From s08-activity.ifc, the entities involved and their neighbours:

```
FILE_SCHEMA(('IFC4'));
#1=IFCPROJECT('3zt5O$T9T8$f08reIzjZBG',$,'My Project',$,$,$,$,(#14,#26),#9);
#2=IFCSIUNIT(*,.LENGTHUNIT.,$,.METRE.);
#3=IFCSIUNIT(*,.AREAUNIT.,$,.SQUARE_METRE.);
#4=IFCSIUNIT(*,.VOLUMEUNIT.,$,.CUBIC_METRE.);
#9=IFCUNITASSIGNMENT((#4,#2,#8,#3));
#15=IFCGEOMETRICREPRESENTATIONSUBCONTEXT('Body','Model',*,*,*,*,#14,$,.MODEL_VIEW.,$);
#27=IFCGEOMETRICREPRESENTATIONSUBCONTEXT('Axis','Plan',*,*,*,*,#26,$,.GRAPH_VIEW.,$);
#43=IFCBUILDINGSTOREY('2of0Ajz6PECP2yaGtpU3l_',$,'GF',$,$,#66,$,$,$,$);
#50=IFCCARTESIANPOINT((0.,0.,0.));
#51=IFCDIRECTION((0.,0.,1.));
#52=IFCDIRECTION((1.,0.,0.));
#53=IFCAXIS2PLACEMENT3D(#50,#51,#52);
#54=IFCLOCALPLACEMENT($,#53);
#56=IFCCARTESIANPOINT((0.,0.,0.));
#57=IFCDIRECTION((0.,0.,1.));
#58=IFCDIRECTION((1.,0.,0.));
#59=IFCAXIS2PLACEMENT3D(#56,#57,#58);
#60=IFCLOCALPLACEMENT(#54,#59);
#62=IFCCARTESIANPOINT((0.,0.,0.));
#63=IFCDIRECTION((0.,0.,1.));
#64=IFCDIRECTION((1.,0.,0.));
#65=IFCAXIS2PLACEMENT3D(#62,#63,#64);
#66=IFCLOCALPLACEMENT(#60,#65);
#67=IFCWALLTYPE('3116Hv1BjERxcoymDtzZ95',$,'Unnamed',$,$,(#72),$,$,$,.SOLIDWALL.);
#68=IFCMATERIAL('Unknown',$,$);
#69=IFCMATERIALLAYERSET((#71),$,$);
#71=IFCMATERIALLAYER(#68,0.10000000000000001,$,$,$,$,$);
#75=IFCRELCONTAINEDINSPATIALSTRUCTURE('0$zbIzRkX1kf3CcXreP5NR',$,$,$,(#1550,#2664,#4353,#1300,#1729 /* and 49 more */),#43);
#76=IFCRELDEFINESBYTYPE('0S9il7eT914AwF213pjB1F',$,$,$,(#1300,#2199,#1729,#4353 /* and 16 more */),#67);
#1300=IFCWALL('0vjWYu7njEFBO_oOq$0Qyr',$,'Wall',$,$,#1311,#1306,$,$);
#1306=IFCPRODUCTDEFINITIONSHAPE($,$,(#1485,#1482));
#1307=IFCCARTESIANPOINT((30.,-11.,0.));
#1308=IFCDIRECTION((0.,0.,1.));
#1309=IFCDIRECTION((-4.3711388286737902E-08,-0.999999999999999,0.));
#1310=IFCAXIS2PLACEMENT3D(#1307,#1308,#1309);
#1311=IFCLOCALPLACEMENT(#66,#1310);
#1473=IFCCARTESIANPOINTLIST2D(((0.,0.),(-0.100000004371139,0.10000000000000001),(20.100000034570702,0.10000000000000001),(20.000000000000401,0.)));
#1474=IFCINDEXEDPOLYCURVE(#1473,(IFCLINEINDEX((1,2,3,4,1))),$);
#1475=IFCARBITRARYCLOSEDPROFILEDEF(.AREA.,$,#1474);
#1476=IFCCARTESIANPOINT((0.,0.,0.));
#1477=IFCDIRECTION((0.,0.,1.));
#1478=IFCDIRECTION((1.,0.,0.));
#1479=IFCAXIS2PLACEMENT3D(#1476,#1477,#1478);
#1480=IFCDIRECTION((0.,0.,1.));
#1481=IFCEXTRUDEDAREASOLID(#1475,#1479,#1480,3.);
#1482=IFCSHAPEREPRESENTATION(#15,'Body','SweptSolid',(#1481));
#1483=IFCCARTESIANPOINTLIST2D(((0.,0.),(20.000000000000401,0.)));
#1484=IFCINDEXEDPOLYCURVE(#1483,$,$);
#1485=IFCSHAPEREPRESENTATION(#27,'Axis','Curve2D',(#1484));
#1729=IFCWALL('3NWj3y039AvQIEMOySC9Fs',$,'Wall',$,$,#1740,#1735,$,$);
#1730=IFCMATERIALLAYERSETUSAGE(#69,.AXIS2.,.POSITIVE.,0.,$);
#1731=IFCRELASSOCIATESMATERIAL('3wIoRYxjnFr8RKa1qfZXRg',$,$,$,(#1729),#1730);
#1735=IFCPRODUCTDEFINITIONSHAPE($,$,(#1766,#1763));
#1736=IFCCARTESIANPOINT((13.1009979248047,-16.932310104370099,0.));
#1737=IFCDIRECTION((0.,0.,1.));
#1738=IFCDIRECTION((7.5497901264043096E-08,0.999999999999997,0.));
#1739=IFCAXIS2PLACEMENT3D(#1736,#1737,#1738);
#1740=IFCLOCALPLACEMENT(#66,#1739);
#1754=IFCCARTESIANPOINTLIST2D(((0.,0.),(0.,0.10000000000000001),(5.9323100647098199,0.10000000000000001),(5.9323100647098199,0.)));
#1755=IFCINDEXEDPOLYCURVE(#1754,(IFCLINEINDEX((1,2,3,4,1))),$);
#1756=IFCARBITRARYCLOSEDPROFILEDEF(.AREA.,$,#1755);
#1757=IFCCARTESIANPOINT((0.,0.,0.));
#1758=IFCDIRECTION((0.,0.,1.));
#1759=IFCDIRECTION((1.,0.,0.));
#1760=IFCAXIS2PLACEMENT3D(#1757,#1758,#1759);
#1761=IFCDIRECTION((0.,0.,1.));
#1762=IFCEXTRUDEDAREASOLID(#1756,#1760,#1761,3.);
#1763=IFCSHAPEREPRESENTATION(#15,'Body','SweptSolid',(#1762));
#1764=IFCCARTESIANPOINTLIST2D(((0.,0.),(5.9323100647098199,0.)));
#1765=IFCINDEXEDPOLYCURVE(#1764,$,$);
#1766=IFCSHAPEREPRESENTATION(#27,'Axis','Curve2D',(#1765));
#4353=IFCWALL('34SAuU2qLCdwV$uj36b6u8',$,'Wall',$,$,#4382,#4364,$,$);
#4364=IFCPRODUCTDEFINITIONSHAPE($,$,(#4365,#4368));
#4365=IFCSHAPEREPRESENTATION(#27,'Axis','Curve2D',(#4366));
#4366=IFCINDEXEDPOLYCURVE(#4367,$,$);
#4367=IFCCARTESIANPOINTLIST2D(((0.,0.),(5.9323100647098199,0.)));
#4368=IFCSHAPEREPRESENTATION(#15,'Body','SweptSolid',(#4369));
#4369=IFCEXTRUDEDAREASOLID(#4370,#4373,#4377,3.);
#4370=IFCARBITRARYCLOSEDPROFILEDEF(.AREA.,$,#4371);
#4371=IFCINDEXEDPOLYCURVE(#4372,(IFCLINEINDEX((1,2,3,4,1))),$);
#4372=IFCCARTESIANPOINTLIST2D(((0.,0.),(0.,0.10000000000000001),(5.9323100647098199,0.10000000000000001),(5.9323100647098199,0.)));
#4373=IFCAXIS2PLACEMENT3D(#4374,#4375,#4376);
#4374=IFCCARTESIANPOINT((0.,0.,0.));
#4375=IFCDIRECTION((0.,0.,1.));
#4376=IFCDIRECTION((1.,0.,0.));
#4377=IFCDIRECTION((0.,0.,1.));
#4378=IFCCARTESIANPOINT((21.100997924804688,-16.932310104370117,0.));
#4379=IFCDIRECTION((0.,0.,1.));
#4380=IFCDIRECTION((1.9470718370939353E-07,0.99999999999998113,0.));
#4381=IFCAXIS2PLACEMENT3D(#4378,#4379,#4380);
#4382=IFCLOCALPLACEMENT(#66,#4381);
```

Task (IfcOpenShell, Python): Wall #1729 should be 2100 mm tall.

```python
import ifcopenshell
import ifcopenshell.geom
import ifcopenshell.util.representation
import ifcopenshell.util.shape
import ifcopenshell.util.unit

model = ifcopenshell.open("s08-activity.ifc")
unit_scale = ifcopenshell.util.unit.calculate_unit_scale(model)
settings = ifcopenshell.geom.settings()


def volume(element):
    """Net volume in cubic metres, openings subtracted."""
    shape = ifcopenshell.geom.create_shape(settings, element)
    return ifcopenshell.util.shape.get_volume(shape.geometry)


wall = model.by_guid("3NWj3y039AvQIEMOySC9Fs")
before = volume(wall)

body = ifcopenshell.util.representation.get_representation(wall, "Model", "Body")
solid = body.Items[0]
old_height = solid.Depth
solid.Depth = 2.1 / unit_scale
after = volume(wall)

print(f"height {old_height:g} -> {solid.Depth:g}, volume {before:.3f} -> {after:.3f} m3")

model.write("s08-activity_edited.ifc")
```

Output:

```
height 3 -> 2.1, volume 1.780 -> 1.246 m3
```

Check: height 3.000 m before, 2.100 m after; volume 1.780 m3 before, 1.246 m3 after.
